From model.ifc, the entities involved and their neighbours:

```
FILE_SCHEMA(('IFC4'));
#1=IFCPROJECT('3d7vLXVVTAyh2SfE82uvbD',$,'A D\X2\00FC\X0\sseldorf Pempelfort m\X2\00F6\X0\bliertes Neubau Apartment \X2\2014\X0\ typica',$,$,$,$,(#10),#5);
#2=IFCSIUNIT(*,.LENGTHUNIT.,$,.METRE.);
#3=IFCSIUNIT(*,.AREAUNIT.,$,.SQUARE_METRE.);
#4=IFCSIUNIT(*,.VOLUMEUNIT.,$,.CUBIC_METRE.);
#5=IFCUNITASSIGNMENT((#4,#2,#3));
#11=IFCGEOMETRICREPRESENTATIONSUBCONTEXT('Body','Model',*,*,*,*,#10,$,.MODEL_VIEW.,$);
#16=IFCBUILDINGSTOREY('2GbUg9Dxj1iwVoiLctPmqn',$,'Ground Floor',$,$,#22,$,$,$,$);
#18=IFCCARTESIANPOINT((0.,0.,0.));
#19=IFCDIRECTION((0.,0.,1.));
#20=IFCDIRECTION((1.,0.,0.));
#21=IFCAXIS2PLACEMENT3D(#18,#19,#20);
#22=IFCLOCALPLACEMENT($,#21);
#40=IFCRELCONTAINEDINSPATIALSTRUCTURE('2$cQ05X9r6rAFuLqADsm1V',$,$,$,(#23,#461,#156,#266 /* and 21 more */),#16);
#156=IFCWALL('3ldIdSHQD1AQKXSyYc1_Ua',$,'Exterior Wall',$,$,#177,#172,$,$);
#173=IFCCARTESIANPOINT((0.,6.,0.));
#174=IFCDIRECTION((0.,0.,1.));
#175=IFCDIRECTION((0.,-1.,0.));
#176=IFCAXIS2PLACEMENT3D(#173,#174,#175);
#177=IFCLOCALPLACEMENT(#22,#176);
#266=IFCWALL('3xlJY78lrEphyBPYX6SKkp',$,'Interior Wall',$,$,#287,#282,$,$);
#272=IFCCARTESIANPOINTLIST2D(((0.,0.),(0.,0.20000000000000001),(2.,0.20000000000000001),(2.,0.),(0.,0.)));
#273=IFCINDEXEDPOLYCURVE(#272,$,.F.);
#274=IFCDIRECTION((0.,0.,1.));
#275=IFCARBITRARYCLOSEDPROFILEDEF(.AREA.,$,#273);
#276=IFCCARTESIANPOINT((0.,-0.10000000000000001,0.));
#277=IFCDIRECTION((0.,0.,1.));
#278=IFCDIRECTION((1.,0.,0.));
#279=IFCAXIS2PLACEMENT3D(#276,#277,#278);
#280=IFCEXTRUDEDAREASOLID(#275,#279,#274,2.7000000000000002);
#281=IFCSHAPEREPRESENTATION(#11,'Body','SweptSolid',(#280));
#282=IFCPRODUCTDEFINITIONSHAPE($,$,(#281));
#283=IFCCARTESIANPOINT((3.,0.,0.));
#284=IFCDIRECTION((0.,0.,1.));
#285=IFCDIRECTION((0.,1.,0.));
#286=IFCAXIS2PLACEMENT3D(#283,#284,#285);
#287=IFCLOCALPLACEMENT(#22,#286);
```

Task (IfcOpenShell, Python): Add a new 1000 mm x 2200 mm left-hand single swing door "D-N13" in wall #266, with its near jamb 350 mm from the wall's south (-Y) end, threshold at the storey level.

```python
import numpy as np
import ifcopenshell
import ifcopenshell.api.feature
import ifcopenshell.api.geometry
import ifcopenshell.api.root
import ifcopenshell.api.spatial
import ifcopenshell.geom
import ifcopenshell.util.element
import ifcopenshell.util.placement
import ifcopenshell.util.representation
import ifcopenshell.util.shape
import ifcopenshell.util.unit

model = ifcopenshell.open("model.ifc")
unit_scale = ifcopenshell.util.unit.calculate_unit_scale(model)
settings = ifcopenshell.geom.settings()


def volume(element):
    """Net volume in cubic metres, openings subtracted."""
    shape = ifcopenshell.geom.create_shape(settings, element)
    return ifcopenshell.util.shape.get_volume(shape.geometry)


wall = model.by_id(266)
storey = ifcopenshell.util.element.get_container(wall, ifc_class="IfcBuildingStorey")
context = ifcopenshell.util.representation.get_context(model, "Model", "Body", "MODEL_VIEW")
before = volume(wall)

width, height, from_end, sill = 1, 2.2, 0.35, 0.0  # metres

# The wall runs along its own X axis, and the end named is its -X end.
wall_shape = ifcopenshell.geom.create_shape(settings, wall)
x, y, z = ifcopenshell.util.shape.get_vertices(wall_shape.geometry).T
start = x.min() + from_end
face, thickness = float(y.min()), float(y.max() - y.min())
wall_matrix = ifcopenshell.util.placement.get_local_placement(wall.ObjectPlacement)
level = ifcopenshell.util.placement.get_local_placement(storey.ObjectPlacement)[2, 3]


def in_wall(x, y):
    """Placement at x, y metres in the wall's axes, at sill height."""
    matrix = wall_matrix.copy()
    matrix[:, 3] = wall_matrix @ np.array([x / unit_scale, y / unit_scale, 0.0, 1.0])
    matrix[2, 3] = level + sill / unit_scale
    return matrix


# Opening: a box that overshoots both wall faces by 50 mm.
opening = ifcopenshell.api.root.create_entity(model, ifc_class="IfcOpeningElement", predefined_type="OPENING")
box = ifcopenshell.api.geometry.add_wall_representation(
    model, context=context, length=width, height=height, thickness=thickness + 0.1
)
ifcopenshell.api.geometry.assign_representation(model, product=opening, representation=box)
ifcopenshell.api.geometry.edit_object_placement(model, product=opening, matrix=in_wall(start, face - 0.05), is_si=False)
ifcopenshell.api.feature.add_feature(model, feature=opening, element=wall)

door = ifcopenshell.api.root.create_entity(model, ifc_class="IfcDoor", name="D-N13", predefined_type="DOOR")
door.OverallWidth, door.OverallHeight = width / unit_scale, height / unit_scale
door.OperationType = "SINGLE_SWING_LEFT"
body = ifcopenshell.api.geometry.add_door_representation(
    model,
    context=context,
    overall_width=door.OverallWidth,
    overall_height=door.OverallHeight,
    operation_type="SINGLE_SWING_LEFT",
    lining_properties={"LiningDepth": thickness / unit_scale, "ThresholdDepth": thickness / unit_scale},
)
ifcopenshell.api.geometry.assign_representation(model, product=door, representation=body)
ifcopenshell.api.spatial.assign_container(model, products=[door], relating_structure=storey)
ifcopenshell.api.feature.add_filling(model, opening=opening, element=door)

# The lining spans the wall, so the door starts at the wall face.
ifcopenshell.api.geometry.edit_object_placement(model, product=door, matrix=in_wall(start, face), is_si=False)

after = volume(wall)

print(f"wall volume {before:.3f} -> {after:.3f} m3")

model.write("model_rev.ifc")
```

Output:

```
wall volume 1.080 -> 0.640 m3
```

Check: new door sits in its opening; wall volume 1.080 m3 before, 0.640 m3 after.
